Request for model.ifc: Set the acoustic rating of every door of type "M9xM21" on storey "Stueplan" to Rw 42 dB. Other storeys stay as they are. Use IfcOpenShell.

First a look at what the model holds.

```python
import ifcopenshell
import ifcopenshell.util.element

model = ifcopenshell.open("model.ifc")
print(model.schema)
storey = next(s for s in model.by_type("IfcBuildingStorey") if s.Name == "Stueplan")
doors = [e for e in ifcopenshell.util.element.get_decomposition(storey) if e.is_a("IfcDoor")]
seen = {}
for e in doors:
    element_type = ifcopenshell.util.element.get_type(e)
    key = (element_type.Name if element_type != e and element_type else None, ifcopenshell.util.element.get_pset(e, "Pset_DoorCommon", "AcousticRating"))
    seen[key] = seen.get(key, 0) + 1
for (name, value), count in sorted(seen.items(), key=str):
    print(count, "x", name, "|", value)
```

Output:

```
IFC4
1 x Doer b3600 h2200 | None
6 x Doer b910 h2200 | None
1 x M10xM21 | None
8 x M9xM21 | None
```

```python
import ifcopenshell
import ifcopenshell.api.pset
import ifcopenshell.util.element

model = ifcopenshell.open("model.ifc")

storey = next(s for s in model.by_type("IfcBuildingStorey") if s.Name == "Stueplan")
doors = [e for e in ifcopenshell.util.element.get_decomposition(storey) if e.is_a("IfcDoor")]

count = 0
for e in doors:
    element_type = ifcopenshell.util.element.get_type(e)
    if element_type in (None, e) or element_type.Name != "M9xM21":
        continue
    # add_pset returns the element's existing set when there is one.
    pset = ifcopenshell.api.pset.add_pset(model, product=e, name="Pset_DoorCommon")
    ifcopenshell.api.pset.edit_pset(model, pset=pset, properties={"AcousticRating": "Rw 42 dB"})
    count += 1

print(count, "doors updated")

model.write("model_rev.ifc")
```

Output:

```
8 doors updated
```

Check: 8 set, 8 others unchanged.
